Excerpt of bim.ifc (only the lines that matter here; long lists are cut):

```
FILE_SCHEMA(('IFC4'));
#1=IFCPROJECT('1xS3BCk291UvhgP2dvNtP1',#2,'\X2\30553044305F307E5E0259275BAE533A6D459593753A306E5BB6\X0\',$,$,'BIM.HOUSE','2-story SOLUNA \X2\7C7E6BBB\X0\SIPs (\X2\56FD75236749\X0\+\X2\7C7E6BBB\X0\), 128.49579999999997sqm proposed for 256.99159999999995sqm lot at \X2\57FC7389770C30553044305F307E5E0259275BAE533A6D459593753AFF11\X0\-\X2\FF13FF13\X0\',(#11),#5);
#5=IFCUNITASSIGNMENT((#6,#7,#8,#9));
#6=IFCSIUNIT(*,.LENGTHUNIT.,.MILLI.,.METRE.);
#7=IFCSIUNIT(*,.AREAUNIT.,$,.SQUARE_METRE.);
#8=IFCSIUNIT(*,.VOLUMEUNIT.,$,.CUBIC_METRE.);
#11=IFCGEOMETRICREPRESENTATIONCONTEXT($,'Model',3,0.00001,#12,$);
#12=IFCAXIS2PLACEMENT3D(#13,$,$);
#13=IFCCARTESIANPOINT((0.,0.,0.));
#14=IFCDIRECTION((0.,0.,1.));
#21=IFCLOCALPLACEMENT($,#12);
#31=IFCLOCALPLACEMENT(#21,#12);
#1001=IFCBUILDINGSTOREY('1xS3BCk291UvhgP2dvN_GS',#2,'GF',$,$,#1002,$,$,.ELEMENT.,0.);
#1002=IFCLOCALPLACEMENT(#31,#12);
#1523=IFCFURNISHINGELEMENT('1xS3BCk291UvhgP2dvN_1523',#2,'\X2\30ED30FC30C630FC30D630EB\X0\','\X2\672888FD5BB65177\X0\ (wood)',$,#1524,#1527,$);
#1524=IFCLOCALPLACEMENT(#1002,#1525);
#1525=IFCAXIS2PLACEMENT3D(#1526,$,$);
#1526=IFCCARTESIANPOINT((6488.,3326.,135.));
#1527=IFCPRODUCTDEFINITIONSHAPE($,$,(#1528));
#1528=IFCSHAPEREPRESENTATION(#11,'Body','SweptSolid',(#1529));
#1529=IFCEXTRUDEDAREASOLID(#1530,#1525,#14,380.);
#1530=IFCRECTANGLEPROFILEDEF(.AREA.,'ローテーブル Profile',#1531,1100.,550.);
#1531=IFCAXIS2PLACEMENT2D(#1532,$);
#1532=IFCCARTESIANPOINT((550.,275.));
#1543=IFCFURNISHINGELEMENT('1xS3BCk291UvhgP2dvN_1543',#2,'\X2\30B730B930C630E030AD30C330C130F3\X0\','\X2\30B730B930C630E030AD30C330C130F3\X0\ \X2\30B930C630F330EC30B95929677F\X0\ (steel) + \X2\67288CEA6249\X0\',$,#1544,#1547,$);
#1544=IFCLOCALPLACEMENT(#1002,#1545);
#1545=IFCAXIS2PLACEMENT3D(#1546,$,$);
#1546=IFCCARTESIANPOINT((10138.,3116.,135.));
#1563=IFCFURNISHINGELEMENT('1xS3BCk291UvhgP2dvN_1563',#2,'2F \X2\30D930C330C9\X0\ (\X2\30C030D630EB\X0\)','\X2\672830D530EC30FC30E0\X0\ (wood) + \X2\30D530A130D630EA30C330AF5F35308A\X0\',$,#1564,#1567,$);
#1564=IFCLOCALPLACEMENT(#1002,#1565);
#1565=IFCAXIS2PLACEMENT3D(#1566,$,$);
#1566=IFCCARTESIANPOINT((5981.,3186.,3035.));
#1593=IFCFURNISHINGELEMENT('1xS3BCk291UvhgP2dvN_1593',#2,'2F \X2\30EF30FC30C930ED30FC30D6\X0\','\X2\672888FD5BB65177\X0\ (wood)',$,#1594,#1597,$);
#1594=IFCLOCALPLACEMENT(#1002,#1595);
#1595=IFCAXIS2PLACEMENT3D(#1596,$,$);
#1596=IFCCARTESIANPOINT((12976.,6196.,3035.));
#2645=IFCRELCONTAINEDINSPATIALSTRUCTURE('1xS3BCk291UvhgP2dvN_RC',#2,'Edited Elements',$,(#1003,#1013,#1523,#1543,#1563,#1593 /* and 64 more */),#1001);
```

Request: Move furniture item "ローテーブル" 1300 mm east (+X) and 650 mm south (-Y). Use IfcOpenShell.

```python
import ifcopenshell
import ifcopenshell.api.geometry
import ifcopenshell.util.placement
import ifcopenshell.util.unit

model = ifcopenshell.open("bim.ifc")
unit_scale = ifcopenshell.util.unit.calculate_unit_scale(model)

item = model.by_guid("1xS3BCk291UvhgP2dvN_1523")
matrix = ifcopenshell.util.placement.get_local_placement(item.ObjectPlacement)
matrix[0, 3] += 1.3 / unit_scale
matrix[1, 3] -= 0.65 / unit_scale
ifcopenshell.api.geometry.edit_object_placement(model, product=item, matrix=matrix, is_si=False)

print(ifcopenshell.util.placement.get_local_placement(item.ObjectPlacement).round(3) + 0.0)

model.write("bim_edited.ifc")
```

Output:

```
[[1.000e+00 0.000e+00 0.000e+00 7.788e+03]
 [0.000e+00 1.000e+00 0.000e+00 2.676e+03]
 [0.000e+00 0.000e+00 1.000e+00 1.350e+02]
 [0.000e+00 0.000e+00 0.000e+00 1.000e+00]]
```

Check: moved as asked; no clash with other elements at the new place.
